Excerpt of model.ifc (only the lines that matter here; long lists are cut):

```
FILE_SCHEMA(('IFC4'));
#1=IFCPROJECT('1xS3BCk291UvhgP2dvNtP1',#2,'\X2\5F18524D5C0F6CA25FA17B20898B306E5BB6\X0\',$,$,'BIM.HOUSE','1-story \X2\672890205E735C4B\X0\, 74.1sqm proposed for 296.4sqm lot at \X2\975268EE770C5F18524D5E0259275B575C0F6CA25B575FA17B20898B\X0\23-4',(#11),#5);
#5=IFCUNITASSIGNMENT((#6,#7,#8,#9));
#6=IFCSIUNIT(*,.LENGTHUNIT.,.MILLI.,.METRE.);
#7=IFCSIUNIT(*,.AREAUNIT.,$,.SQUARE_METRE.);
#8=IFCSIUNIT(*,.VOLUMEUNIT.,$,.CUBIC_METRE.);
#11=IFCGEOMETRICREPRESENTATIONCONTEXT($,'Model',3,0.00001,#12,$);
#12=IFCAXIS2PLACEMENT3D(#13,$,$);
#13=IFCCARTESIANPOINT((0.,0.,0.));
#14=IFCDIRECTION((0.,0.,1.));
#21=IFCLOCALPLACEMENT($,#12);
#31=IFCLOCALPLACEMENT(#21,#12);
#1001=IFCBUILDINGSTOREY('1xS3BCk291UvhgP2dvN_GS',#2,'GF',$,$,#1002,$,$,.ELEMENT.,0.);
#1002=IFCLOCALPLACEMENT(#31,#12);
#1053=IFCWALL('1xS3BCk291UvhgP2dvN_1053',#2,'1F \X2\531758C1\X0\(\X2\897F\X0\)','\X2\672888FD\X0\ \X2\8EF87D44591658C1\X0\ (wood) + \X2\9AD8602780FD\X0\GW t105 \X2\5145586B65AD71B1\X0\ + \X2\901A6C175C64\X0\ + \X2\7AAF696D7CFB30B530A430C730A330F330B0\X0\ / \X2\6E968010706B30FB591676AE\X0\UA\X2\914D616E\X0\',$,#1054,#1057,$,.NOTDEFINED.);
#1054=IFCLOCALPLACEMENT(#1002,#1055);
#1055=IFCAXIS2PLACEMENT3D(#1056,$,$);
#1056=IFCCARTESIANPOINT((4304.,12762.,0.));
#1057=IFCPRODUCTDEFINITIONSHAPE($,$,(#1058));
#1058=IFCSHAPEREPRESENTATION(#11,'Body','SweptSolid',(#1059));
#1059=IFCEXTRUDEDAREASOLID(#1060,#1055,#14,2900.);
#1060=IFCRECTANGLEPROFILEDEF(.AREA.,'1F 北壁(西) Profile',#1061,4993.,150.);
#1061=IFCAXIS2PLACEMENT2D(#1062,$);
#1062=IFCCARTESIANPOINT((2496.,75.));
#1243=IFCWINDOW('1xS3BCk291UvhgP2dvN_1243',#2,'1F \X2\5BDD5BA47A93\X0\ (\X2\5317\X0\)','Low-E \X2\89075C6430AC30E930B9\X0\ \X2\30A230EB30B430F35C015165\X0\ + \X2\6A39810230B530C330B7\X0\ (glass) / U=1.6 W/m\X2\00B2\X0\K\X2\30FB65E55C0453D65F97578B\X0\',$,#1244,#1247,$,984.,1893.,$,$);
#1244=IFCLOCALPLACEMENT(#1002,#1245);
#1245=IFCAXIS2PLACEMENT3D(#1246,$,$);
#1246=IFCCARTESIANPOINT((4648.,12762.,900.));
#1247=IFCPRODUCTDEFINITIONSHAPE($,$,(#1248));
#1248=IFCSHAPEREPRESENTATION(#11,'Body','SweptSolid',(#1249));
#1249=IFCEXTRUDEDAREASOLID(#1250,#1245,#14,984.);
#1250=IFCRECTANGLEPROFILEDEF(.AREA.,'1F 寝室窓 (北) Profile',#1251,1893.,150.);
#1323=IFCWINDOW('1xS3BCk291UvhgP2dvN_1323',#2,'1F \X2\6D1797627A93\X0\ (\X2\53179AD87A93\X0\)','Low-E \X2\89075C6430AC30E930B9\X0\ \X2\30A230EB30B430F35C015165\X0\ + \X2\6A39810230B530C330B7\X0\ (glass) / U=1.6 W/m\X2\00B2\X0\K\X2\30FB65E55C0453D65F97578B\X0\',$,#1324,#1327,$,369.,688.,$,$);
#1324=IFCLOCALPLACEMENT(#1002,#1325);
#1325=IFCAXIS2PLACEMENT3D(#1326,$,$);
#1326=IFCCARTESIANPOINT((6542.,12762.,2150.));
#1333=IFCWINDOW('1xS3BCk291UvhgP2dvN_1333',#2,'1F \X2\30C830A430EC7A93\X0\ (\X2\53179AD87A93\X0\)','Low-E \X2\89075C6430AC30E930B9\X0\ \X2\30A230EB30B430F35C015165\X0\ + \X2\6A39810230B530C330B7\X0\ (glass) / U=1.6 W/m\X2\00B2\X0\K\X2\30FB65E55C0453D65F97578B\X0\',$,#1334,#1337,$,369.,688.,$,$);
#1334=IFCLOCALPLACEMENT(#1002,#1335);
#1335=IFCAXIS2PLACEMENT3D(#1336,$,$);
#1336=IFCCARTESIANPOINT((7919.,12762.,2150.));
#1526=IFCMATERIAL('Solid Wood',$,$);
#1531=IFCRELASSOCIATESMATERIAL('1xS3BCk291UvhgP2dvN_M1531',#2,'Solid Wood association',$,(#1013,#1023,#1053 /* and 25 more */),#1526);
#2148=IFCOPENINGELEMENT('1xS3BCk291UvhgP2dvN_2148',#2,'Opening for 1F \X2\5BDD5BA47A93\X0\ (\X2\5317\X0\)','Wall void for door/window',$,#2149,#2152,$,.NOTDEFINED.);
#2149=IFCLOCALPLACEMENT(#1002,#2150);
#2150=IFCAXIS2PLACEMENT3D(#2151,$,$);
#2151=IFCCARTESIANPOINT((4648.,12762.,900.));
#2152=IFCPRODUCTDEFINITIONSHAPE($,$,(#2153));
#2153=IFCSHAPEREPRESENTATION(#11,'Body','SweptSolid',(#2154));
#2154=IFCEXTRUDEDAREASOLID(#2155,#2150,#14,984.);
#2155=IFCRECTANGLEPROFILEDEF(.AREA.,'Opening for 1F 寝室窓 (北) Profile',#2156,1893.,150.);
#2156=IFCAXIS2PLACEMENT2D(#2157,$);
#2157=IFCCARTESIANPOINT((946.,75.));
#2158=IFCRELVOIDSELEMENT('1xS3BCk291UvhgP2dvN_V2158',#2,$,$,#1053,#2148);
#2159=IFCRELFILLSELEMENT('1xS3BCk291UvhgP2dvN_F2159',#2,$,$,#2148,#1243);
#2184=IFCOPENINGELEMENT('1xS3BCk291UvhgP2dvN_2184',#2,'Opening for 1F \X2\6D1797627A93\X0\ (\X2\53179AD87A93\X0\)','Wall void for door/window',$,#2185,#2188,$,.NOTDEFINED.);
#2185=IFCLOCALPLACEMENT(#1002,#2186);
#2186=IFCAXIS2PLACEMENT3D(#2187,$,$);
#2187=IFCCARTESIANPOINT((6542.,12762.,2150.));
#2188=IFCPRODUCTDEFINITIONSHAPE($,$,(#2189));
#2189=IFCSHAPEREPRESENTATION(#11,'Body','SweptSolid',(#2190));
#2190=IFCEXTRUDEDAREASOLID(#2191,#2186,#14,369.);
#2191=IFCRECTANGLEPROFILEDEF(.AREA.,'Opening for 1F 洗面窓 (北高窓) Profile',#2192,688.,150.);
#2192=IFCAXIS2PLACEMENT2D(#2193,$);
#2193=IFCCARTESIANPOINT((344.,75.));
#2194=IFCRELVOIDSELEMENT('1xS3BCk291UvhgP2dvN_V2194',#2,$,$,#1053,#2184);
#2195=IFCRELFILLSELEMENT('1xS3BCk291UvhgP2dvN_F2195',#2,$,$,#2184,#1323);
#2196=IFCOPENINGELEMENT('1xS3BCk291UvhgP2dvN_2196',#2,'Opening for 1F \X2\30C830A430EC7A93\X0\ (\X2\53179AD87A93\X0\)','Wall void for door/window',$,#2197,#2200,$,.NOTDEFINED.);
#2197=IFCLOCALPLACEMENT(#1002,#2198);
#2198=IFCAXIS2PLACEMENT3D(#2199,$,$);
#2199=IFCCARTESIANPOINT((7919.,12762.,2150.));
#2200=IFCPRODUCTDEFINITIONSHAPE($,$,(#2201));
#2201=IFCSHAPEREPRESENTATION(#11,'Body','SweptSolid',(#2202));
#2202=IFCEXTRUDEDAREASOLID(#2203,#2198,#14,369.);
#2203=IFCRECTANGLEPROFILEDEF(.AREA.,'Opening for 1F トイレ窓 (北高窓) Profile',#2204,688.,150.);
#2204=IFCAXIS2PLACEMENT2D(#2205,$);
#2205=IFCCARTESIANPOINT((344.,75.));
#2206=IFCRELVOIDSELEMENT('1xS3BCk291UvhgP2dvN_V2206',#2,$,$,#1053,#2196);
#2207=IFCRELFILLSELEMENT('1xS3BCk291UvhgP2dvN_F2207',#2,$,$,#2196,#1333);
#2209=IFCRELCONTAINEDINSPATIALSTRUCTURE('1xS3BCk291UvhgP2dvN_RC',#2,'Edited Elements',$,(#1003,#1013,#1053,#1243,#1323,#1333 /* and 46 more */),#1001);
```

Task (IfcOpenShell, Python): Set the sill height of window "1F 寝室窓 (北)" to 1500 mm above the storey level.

```python
import numpy as np
import ifcopenshell
import ifcopenshell.api.geometry
import ifcopenshell.geom
import ifcopenshell.util.element
import ifcopenshell.util.placement
import ifcopenshell.util.shape
import ifcopenshell.util.unit

model = ifcopenshell.open("model.ifc")
unit_scale = ifcopenshell.util.unit.calculate_unit_scale(model)

window = model.by_guid("1xS3BCk291UvhgP2dvN_1243")
opening = window.FillsVoids[0].RelatingOpeningElement
storey = ifcopenshell.util.element.get_container(window, ifc_class="IfcBuildingStorey")
level = ifcopenshell.util.placement.get_local_placement(storey.ObjectPlacement)[2, 3]

# The opening's origin need not be at the sill, so measure its lowest point.
shape = ifcopenshell.geom.create_shape(ifcopenshell.geom.settings(), opening)
bottom = ifcopenshell.util.shape.get_shape_bottom_elevation(shape, shape.geometry) / unit_scale
dz = level + 1.5 / unit_scale - bottom

shift = np.array([0.0, 0.0, dz])
# The window is not placed relative to its opening, so move both.
for product in (opening, window):
    matrix = ifcopenshell.util.placement.get_local_placement(product.ObjectPlacement)
    matrix[:3, 3] += shift
    ifcopenshell.api.geometry.edit_object_placement(model, product=product, matrix=matrix, is_si=False)

print(f"moved by {dz * unit_scale:+.3f} m")

model.write("model_v2.ifc")
```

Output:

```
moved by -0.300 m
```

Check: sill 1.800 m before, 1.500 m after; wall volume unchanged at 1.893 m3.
